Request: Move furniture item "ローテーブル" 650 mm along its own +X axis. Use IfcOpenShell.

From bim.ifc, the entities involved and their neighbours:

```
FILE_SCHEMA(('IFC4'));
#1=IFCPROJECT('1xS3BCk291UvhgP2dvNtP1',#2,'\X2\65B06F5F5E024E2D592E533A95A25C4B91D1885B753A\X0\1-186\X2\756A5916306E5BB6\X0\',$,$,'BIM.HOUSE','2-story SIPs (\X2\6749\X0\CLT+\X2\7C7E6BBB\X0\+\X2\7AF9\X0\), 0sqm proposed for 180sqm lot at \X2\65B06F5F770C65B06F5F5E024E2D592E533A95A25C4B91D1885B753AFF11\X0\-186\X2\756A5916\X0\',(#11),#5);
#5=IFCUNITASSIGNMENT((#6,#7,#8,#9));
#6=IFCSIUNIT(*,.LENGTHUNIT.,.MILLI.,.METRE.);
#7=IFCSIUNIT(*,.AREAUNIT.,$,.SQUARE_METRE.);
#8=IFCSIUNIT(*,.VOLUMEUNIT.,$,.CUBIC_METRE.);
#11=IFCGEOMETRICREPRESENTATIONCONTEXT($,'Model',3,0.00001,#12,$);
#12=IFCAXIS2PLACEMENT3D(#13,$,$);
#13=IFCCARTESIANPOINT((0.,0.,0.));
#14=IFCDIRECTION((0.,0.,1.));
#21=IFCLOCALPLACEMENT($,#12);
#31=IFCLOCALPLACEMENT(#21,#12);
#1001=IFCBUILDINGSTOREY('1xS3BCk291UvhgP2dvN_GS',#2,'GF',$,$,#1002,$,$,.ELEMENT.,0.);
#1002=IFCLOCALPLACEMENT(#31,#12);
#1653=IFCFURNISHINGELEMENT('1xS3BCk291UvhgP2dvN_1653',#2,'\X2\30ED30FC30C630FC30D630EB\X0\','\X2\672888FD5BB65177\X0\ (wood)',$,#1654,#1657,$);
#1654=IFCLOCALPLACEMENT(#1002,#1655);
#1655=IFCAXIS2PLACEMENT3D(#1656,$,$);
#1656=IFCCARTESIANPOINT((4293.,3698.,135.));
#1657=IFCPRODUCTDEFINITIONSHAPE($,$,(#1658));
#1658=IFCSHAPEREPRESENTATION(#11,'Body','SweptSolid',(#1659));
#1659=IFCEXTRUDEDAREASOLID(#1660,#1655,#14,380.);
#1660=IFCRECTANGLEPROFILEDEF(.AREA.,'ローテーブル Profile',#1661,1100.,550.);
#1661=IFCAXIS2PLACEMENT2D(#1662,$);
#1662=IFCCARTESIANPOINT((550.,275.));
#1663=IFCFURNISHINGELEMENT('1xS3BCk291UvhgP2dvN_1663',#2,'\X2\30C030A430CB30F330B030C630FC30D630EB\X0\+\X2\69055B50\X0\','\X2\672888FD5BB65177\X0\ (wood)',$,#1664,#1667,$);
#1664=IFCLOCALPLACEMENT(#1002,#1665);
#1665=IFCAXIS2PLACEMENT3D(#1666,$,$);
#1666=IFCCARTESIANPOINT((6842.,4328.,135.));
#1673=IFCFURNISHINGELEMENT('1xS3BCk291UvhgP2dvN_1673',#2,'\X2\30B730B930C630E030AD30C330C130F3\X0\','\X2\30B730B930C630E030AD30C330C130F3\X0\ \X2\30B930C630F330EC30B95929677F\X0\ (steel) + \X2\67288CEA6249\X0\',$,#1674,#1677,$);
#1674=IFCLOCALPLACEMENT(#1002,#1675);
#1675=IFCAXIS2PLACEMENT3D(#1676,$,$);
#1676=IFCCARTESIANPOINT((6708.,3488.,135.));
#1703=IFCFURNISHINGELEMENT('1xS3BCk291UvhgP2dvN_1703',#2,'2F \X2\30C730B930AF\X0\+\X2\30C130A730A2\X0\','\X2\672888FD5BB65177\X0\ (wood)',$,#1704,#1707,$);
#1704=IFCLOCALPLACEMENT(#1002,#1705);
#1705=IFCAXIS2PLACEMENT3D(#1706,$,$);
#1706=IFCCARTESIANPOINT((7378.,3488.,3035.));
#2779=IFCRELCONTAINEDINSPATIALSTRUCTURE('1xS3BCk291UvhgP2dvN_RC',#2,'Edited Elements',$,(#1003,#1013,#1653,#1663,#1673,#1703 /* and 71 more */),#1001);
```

```python
import ifcopenshell
import ifcopenshell.api.geometry
import ifcopenshell.util.placement
import ifcopenshell.util.unit

model = ifcopenshell.open("bim.ifc")
unit_scale = ifcopenshell.util.unit.calculate_unit_scale(model)

item = model.by_id(1653)
matrix = ifcopenshell.util.placement.get_local_placement(item.ObjectPlacement)
matrix[:3, 3] += matrix[:3, 0] * 0.65 / unit_scale
ifcopenshell.api.geometry.edit_object_placement(model, product=item, matrix=matrix, is_si=False)

print(ifcopenshell.util.placement.get_local_placement(item.ObjectPlacement).round(3) + 0.0)

model.write("bim_updated.ifc")
```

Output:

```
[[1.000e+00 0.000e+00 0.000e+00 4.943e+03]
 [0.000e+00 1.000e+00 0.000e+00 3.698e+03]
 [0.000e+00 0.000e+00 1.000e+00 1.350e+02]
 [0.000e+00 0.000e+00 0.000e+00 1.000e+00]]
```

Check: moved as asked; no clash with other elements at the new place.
